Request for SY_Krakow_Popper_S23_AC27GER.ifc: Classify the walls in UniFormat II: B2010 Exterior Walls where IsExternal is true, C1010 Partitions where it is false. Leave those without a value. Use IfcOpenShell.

First a look at what the model holds.

```python
import ifcopenshell
import ifcopenshell.util.element

model = ifcopenshell.open("SY_Krakow_Popper_S23_AC27GER.ifc")
print(model.schema)
print("classifications:", [c.Name for c in model.by_type("IfcClassification")])
values = [ifcopenshell.util.element.get_pset(e, "Pset_WallCommon", "IsExternal") for e in model.by_type("IfcWall")]
for value in (True, False, None):
    print("IsExternal", value, values.count(value))
```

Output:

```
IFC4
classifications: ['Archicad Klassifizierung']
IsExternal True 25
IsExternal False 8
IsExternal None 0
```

```python
import ifcopenshell
import ifcopenshell.api.classification
import ifcopenshell.util.element

model = ifcopenshell.open("SY_Krakow_Popper_S23_AC27GER.ifc")

system = ifcopenshell.api.classification.add_classification(model, classification="UniFormat II")

walls = model.by_type("IfcWall")
external = {e: ifcopenshell.util.element.get_pset(e, "Pset_WallCommon", "IsExternal") for e in walls}
for flag, code, name in ((True, "B2010", "Exterior Walls"), (False, "C1010", "Partitions")):
    products = [e for e in walls if external[e] is flag]
    ifcopenshell.api.classification.add_reference(
        model, products=products, classification=system, identification=code, name=name
    )
    print(code, len(products))

model.write("SY_Krakow_Popper_S23_AC27GER_edited.ifc")
```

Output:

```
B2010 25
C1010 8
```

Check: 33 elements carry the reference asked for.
